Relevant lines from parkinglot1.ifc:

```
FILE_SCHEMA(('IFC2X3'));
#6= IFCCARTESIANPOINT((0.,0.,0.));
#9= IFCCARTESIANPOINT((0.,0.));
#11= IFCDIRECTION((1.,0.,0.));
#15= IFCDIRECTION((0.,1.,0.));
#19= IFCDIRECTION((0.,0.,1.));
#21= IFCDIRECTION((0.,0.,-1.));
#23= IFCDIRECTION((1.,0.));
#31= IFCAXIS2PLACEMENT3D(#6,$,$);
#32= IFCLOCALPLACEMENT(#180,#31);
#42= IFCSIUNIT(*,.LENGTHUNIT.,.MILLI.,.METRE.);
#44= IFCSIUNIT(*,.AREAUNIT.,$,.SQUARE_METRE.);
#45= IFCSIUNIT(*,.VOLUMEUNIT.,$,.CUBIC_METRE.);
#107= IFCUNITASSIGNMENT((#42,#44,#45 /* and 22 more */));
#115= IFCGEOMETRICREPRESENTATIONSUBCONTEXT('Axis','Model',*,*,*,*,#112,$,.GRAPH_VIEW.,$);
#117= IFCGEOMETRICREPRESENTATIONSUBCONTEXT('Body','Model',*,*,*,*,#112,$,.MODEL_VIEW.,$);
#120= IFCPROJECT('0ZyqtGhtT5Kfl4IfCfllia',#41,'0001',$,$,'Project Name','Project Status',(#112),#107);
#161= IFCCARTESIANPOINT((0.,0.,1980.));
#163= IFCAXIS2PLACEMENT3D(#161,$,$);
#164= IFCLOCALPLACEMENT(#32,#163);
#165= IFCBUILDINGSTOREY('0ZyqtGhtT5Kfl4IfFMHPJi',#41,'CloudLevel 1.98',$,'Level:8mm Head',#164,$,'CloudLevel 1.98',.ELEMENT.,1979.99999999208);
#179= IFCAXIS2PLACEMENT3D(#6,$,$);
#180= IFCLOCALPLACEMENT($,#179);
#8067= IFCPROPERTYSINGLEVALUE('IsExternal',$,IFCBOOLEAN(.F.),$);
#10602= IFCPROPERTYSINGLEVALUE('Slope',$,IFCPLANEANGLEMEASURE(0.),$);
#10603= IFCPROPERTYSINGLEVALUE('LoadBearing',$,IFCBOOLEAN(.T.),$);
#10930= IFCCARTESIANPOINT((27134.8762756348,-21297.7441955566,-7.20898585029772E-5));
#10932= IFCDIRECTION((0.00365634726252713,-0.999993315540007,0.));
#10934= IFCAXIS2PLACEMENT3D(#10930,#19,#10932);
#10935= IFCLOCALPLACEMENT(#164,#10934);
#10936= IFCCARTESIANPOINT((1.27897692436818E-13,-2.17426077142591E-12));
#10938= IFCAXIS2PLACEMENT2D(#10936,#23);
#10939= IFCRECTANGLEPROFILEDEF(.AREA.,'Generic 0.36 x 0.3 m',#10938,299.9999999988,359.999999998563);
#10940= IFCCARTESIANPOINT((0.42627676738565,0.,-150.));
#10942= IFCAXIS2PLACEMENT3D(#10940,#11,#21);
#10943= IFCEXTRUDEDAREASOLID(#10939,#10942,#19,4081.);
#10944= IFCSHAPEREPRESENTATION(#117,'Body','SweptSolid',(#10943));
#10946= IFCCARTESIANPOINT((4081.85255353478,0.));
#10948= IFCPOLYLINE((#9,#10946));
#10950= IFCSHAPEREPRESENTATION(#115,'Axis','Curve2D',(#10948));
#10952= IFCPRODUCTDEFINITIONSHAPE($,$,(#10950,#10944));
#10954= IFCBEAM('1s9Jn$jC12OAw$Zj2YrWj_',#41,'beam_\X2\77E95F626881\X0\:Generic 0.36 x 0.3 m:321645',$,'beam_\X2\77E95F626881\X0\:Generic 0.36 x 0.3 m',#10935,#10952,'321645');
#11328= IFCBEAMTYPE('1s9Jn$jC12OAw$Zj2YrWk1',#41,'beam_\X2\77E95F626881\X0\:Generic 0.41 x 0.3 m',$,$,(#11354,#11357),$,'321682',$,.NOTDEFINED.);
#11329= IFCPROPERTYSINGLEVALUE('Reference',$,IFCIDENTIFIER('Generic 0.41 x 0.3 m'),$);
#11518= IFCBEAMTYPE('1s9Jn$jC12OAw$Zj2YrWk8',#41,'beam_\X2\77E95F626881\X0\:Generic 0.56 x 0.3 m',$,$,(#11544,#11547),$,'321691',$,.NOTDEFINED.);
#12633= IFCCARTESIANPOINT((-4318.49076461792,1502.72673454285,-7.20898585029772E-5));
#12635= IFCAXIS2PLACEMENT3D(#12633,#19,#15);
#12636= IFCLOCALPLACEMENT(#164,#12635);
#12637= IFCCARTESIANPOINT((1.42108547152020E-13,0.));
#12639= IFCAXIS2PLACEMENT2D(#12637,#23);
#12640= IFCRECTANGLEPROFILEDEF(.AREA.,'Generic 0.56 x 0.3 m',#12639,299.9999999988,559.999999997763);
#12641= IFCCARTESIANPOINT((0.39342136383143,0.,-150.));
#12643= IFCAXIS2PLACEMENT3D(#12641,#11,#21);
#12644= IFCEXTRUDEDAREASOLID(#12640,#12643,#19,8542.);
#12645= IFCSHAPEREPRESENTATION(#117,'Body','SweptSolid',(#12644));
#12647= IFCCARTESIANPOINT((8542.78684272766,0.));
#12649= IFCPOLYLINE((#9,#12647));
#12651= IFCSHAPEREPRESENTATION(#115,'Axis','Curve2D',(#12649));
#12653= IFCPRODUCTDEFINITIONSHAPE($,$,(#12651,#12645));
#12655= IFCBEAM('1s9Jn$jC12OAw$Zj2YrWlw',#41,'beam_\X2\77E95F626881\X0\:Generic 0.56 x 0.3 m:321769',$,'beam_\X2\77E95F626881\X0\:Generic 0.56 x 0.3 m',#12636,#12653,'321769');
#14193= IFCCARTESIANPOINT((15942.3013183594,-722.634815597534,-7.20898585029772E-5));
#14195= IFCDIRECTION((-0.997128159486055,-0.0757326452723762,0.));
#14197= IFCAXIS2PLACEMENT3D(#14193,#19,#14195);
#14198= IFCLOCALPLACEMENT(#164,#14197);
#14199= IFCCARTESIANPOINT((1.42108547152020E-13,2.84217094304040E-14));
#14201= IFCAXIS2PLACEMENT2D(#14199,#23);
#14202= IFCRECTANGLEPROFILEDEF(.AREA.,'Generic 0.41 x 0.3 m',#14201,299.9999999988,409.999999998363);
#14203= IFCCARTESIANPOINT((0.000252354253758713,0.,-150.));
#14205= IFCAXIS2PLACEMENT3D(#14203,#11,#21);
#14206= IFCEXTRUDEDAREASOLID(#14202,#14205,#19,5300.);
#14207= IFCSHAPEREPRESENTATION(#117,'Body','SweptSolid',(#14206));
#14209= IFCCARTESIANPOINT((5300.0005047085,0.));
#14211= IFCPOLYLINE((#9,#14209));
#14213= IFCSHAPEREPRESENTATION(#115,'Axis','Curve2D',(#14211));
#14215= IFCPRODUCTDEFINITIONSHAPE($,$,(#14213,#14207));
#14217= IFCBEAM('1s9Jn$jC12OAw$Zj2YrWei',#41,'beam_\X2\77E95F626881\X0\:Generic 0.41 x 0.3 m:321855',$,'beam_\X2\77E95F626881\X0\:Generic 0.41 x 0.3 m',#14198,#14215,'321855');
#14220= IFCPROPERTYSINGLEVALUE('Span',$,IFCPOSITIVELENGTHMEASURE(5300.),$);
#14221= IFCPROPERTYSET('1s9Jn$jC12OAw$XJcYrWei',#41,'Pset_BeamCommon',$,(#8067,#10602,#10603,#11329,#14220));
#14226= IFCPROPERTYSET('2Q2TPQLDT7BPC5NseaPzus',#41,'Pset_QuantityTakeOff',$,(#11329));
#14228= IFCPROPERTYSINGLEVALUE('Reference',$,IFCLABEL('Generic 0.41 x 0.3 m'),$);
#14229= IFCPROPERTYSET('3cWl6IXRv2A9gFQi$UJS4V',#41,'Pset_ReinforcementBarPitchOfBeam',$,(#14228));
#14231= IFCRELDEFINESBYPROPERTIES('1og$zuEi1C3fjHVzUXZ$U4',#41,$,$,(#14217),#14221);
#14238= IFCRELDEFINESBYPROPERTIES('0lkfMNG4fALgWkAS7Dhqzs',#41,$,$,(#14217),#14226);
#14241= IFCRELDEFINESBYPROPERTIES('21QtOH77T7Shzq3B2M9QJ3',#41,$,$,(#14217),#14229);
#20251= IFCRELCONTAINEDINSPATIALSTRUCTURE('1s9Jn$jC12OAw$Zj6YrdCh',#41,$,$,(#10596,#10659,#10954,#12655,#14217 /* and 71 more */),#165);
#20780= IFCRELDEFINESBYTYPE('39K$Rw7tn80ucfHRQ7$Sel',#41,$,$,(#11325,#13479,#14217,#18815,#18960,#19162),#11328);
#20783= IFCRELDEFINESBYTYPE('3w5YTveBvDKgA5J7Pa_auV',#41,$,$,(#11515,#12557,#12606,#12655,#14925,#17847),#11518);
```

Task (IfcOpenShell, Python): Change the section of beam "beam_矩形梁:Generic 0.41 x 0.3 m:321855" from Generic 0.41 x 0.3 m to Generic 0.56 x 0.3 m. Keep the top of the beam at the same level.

```python
import ifcopenshell
import ifcopenshell.api.pset
import ifcopenshell.api.type
import ifcopenshell.util.element
import ifcopenshell.util.representation

model = ifcopenshell.open("parkinglot1.ifc")

member = model.by_guid("1s9Jn$jC12OAw$Zj2YrWei")
source = next(p for p in model.by_type("IfcRectangleProfileDef") if p.ProfileName == "Generic 0.56 x 0.3 m")

body = ifcopenshell.util.representation.get_representation(member, "Model", "Body")
solid = body.Items[0]
old_profile = solid.SweptArea

# Copy the section's sizes but keep this member's own profile position.
profile = ifcopenshell.util.element.copy(model, source)
# Profiles are centred, so shift by half the change in depth to hold the top.
shift = (old_profile.XDim - profile.XDim) / 2
x, y = old_profile.Position.Location.Coordinates
up = (-1.0, 0.0)  # upwards, in the solid's own plane
location = model.createIfcCartesianPoint((x + up[0] * shift, y + up[1] * shift))
profile.Position = model.createIfcAxis2Placement2D(location, old_profile.Position.RefDirection)
solid.SweptArea = profile
if not model.get_total_inverses(old_profile):
    ifcopenshell.util.element.remove_deep2(model, old_profile)

new_type = model.by_guid("1s9Jn$jC12OAw$Zj2YrWk8")
ifcopenshell.api.type.assign_type(
    model, related_objects=[member], relating_type=new_type, should_map_representations=False
)
member.Name = member.Name.replace("Generic 0.41 x 0.3 m", "Generic 0.56 x 0.3 m")
member.ObjectType = "beam_矩形梁:Generic 0.56 x 0.3 m"
pset = model.by_id(ifcopenshell.util.element.get_pset(member, "Pset_BeamCommon", should_inherit=False)["id"])
ifcopenshell.api.pset.edit_pset(model, pset=pset, properties={"Reference": "Generic 0.56 x 0.3 m"})
pset = model.by_id(ifcopenshell.util.element.get_pset(member, "Pset_QuantityTakeOff", should_inherit=False)["id"])
ifcopenshell.api.pset.edit_pset(model, pset=pset, properties={"Reference": "Generic 0.56 x 0.3 m"})
pset = model.by_id(ifcopenshell.util.element.get_pset(member, "Pset_ReinforcementBarPitchOfBeam", should_inherit=False)["id"])
ifcopenshell.api.pset.edit_pset(model, pset=pset, properties={"Reference": "Generic 0.56 x 0.3 m"})

print(solid.SweptArea)

model.write("parkinglot1-out.ifc")
```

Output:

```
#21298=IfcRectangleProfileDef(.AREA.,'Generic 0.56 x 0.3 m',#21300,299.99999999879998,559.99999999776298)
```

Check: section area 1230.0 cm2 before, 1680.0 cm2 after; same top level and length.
